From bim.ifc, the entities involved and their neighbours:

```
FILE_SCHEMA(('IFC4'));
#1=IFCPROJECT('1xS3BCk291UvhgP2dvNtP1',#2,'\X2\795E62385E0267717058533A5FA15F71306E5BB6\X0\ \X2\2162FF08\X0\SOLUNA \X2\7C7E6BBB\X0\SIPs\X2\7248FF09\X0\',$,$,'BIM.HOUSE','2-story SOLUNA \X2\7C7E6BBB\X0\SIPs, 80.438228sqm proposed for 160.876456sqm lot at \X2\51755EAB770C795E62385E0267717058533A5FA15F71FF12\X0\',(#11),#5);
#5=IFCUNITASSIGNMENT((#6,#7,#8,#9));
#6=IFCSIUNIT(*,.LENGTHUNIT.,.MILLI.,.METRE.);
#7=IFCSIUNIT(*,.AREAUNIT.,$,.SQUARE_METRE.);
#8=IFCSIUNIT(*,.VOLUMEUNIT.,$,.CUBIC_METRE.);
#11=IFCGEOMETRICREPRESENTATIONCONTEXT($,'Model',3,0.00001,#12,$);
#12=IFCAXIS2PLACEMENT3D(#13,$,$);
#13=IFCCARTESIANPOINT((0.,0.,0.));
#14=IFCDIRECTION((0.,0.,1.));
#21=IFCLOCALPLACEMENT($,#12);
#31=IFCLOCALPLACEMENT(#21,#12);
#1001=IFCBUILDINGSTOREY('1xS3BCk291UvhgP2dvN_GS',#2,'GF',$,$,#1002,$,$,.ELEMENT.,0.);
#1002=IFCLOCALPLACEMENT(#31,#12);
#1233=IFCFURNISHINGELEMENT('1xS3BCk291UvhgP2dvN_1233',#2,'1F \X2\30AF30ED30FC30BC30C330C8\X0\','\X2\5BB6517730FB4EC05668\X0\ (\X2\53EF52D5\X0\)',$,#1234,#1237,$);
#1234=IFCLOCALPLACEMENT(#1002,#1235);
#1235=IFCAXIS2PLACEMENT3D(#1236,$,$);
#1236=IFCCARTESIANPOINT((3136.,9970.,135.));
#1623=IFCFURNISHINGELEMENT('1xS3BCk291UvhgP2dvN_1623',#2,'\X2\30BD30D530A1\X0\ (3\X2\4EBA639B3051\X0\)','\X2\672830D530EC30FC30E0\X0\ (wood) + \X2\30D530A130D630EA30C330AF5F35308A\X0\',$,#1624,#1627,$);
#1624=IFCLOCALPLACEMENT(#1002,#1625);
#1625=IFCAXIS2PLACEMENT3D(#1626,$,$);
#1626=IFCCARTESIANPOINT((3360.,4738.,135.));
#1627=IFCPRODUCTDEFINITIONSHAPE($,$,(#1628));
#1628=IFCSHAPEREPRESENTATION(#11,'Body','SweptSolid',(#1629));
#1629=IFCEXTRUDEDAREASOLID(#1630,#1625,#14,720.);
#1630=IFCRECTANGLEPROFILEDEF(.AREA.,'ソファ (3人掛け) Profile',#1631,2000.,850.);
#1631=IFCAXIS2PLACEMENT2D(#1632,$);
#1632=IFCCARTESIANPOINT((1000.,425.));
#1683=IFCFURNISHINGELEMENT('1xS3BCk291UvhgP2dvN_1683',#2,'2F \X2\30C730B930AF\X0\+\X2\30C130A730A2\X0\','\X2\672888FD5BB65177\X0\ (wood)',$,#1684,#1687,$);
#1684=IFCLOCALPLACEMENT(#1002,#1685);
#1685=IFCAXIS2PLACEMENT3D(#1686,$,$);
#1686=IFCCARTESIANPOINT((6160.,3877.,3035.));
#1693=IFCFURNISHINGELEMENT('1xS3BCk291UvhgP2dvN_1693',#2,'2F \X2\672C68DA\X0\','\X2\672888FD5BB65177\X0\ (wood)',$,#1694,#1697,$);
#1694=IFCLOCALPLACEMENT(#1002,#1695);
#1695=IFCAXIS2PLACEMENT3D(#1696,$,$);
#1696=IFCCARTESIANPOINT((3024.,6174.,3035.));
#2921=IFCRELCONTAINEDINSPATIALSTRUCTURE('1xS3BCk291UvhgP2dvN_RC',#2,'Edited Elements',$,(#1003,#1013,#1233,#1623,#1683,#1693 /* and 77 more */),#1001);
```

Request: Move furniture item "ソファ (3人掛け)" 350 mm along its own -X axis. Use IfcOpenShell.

```python
import ifcopenshell
import ifcopenshell.api.geometry
import ifcopenshell.util.placement
import ifcopenshell.util.unit

model = ifcopenshell.open("bim.ifc")
unit_scale = ifcopenshell.util.unit.calculate_unit_scale(model)

item = model.by_guid("1xS3BCk291UvhgP2dvN_1623")
matrix = ifcopenshell.util.placement.get_local_placement(item.ObjectPlacement)
matrix[:3, 3] -= matrix[:3, 0] * 0.35 / unit_scale
ifcopenshell.api.geometry.edit_object_placement(model, product=item, matrix=matrix, is_si=False)

print(ifcopenshell.util.placement.get_local_placement(item.ObjectPlacement).round(3) + 0.0)

model.write("bim_rev.ifc")
```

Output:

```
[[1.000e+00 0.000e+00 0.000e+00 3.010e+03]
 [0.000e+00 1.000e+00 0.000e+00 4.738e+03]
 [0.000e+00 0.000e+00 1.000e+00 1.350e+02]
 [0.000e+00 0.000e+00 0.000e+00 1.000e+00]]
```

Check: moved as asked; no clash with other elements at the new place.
